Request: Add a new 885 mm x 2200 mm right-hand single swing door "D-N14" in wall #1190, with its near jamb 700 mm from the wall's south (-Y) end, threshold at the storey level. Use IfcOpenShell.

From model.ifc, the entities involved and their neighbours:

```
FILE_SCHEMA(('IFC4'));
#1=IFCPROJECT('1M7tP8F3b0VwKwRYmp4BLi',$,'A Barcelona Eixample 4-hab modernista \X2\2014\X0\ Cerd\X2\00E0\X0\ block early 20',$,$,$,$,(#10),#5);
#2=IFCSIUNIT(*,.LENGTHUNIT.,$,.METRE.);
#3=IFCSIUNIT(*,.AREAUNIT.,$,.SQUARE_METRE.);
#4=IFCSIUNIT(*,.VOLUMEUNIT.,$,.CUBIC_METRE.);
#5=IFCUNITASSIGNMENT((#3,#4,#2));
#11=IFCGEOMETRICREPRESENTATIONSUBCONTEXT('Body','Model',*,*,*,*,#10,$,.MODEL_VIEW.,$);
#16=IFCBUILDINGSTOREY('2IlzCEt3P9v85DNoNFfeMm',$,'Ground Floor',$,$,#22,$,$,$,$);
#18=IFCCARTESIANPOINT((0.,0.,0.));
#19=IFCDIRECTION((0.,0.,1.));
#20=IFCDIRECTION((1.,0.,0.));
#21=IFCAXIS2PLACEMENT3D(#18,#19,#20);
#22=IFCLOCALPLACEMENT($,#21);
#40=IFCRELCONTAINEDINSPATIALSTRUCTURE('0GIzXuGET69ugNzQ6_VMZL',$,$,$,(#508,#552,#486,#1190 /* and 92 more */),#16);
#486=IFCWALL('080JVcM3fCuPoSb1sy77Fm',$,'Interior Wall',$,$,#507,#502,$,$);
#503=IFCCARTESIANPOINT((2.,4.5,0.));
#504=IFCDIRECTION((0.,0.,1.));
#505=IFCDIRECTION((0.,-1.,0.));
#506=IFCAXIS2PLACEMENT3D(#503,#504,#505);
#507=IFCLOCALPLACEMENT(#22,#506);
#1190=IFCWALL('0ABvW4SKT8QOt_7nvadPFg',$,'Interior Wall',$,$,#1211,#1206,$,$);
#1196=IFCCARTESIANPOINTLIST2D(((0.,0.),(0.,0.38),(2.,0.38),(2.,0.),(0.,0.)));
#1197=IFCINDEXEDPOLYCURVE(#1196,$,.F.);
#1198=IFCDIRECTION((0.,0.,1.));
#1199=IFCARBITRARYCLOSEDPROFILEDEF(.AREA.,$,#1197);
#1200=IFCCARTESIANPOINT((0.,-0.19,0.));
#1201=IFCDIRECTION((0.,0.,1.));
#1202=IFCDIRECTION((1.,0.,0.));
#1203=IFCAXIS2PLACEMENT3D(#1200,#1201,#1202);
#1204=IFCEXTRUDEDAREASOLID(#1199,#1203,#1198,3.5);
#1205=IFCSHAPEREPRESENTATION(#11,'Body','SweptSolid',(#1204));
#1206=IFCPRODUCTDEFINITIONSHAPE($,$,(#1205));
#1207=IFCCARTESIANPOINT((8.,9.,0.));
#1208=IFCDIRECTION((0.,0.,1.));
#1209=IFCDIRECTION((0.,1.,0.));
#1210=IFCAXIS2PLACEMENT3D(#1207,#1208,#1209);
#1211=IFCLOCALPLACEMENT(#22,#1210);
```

```python
import numpy as np
import ifcopenshell
import ifcopenshell.api.feature
import ifcopenshell.api.geometry
import ifcopenshell.api.root
import ifcopenshell.api.spatial
import ifcopenshell.geom
import ifcopenshell.util.element
import ifcopenshell.util.placement
import ifcopenshell.util.representation
import ifcopenshell.util.shape
import ifcopenshell.util.unit

model = ifcopenshell.open("model.ifc")
unit_scale = ifcopenshell.util.unit.calculate_unit_scale(model)
settings = ifcopenshell.geom.settings()


def volume(element):
    """Net volume in cubic metres, openings subtracted."""
    shape = ifcopenshell.geom.create_shape(settings, element)
    return ifcopenshell.util.shape.get_volume(shape.geometry)


wall = model.by_id(1190)
storey = ifcopenshell.util.element.get_container(wall, ifc_class="IfcBuildingStorey")
context = ifcopenshell.util.representation.get_context(model, "Model", "Body", "MODEL_VIEW")
before = volume(wall)

width, height, from_end, sill = 0.885, 2.2, 0.7, 0.0  # metres

# The wall runs along its own X axis, and the end named is its -X end.
wall_shape = ifcopenshell.geom.create_shape(settings, wall)
x, y, z = ifcopenshell.util.shape.get_vertices(wall_shape.geometry).T
start = x.min() + from_end
face, thickness = float(y.min()), float(y.max() - y.min())
wall_matrix = ifcopenshell.util.placement.get_local_placement(wall.ObjectPlacement)
level = ifcopenshell.util.placement.get_local_placement(storey.ObjectPlacement)[2, 3]


def in_wall(x, y):
    """Placement at x, y metres in the wall's axes, at sill height."""
    matrix = wall_matrix.copy()
    matrix[:, 3] = wall_matrix @ np.array([x / unit_scale, y / unit_scale, 0.0, 1.0])
    matrix[2, 3] = level + sill / unit_scale
    return matrix


# Opening: a box that overshoots both wall faces by 50 mm.
opening = ifcopenshell.api.root.create_entity(model, ifc_class="IfcOpeningElement", predefined_type="OPENING")
box = ifcopenshell.api.geometry.add_wall_representation(
    model, context=context, length=width, height=height, thickness=thickness + 0.1
)
ifcopenshell.api.geometry.assign_representation(model, product=opening, representation=box)
ifcopenshell.api.geometry.edit_object_placement(model, product=opening, matrix=in_wall(start, face - 0.05), is_si=False)
ifcopenshell.api.feature.add_feature(model, feature=opening, element=wall)

door = ifcopenshell.api.root.create_entity(model, ifc_class="IfcDoor", name="D-N14", predefined_type="DOOR")
door.OverallWidth, door.OverallHeight = width / unit_scale, height / unit_scale
door.OperationType = "SINGLE_SWING_RIGHT"
body = ifcopenshell.api.geometry.add_door_representation(
    model,
    context=context,
    overall_width=door.OverallWidth,
    overall_height=door.OverallHeight,
    operation_type="SINGLE_SWING_RIGHT",
    lining_properties={"LiningDepth": thickness / unit_scale, "ThresholdDepth": thickness / unit_scale},
)
ifcopenshell.api.geometry.assign_representation(model, product=door, representation=body)
ifcopenshell.api.spatial.assign_container(model, products=[door], relating_structure=storey)
ifcopenshell.api.feature.add_filling(model, opening=opening, element=door)

# The lining spans the wall, so the door starts at the wall face.
ifcopenshell.api.geometry.edit_object_placement(model, product=door, matrix=in_wall(start, face), is_si=False)

after = volume(wall)

print(f"wall volume {before:.3f} -> {after:.3f} m3")

model.write("model_updated.ifc")
```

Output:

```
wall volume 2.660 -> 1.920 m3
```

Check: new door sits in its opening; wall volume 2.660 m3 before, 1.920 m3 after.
